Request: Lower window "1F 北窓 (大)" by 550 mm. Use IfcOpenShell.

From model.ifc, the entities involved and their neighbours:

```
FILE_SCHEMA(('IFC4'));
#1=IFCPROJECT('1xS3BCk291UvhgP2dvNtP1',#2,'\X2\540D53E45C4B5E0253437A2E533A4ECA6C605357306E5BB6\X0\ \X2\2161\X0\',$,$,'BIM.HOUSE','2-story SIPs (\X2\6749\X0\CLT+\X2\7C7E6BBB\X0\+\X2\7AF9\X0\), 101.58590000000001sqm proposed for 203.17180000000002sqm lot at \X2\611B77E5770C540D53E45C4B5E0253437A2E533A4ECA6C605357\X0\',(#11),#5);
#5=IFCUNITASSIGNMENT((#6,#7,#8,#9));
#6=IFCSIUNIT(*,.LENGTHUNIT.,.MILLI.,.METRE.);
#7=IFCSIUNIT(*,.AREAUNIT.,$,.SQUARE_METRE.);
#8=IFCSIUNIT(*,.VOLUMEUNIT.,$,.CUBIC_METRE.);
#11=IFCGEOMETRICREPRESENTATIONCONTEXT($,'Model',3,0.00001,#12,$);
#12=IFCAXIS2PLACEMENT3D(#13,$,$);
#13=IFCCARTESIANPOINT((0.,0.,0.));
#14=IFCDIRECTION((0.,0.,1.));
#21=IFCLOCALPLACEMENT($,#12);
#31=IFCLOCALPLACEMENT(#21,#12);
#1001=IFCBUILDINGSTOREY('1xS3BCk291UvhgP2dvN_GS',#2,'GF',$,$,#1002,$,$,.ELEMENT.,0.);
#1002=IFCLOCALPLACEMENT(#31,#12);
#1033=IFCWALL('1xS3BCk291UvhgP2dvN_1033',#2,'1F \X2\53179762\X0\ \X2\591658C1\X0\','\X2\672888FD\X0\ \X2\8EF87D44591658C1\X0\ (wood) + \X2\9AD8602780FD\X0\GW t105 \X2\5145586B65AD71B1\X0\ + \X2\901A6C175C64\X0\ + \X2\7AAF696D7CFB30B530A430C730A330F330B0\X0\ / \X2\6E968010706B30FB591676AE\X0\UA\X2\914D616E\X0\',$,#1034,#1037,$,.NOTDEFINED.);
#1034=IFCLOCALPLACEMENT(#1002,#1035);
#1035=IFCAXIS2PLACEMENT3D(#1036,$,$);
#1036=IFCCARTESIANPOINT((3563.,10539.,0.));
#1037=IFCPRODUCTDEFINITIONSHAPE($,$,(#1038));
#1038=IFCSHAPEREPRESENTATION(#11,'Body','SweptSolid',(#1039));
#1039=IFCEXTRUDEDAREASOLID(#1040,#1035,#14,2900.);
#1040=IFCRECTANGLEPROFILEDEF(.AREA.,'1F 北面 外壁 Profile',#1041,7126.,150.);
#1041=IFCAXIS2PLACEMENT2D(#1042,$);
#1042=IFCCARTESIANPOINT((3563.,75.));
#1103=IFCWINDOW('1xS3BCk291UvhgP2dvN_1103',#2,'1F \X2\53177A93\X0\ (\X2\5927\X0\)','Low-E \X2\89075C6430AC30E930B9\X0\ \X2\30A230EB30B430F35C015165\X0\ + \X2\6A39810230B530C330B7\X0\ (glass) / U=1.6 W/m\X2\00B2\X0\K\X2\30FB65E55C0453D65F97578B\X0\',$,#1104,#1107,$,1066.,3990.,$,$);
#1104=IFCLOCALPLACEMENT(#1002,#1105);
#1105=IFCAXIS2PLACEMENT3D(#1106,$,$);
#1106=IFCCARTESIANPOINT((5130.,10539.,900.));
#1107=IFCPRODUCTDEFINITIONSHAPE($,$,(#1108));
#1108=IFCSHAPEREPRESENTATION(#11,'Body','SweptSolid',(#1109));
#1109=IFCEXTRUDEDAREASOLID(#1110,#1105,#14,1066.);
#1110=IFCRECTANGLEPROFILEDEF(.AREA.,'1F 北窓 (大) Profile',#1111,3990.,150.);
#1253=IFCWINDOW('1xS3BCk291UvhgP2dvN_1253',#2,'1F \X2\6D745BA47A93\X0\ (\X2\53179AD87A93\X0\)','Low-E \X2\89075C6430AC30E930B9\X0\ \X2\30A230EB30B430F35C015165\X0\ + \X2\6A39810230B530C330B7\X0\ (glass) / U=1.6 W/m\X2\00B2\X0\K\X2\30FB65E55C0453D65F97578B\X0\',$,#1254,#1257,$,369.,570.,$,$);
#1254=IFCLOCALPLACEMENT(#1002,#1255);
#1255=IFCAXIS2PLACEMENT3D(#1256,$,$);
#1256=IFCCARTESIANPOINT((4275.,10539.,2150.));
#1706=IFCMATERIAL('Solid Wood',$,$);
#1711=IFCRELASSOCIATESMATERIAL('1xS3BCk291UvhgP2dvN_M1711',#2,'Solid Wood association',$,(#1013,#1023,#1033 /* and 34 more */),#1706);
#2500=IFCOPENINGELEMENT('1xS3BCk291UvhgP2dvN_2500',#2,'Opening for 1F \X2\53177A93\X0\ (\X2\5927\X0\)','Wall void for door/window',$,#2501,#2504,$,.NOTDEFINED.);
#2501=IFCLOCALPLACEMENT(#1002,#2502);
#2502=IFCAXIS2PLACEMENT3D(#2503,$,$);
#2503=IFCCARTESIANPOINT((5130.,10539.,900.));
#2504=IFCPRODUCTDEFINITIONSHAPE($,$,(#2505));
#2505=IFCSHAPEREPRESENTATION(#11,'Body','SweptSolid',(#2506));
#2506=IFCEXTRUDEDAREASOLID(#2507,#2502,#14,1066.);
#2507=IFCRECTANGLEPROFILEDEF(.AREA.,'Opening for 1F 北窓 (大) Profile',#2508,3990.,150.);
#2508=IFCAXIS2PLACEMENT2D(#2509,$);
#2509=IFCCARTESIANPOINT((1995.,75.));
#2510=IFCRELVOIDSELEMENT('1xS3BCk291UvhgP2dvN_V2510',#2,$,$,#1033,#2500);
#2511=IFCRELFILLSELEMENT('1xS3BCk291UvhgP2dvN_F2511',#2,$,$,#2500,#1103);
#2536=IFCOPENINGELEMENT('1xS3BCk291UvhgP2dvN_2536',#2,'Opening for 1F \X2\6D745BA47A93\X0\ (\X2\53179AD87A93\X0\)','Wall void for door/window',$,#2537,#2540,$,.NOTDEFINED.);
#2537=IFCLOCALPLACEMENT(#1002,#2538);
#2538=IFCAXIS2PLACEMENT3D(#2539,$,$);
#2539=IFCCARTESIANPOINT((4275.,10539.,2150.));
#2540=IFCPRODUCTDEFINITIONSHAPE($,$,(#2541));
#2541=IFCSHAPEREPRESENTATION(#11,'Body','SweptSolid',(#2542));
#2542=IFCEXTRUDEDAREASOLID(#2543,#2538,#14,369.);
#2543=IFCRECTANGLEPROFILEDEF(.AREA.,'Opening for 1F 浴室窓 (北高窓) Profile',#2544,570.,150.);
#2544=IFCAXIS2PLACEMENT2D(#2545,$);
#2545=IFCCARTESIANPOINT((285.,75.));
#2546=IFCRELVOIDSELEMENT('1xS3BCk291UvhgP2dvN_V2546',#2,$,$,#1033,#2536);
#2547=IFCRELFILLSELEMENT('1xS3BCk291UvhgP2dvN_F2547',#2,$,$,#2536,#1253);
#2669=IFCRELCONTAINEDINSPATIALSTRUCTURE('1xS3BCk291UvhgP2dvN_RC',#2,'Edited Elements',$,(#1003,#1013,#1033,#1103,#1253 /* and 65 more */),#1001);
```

```python
import numpy as np
import ifcopenshell
import ifcopenshell.api.geometry
import ifcopenshell.util.placement
import ifcopenshell.util.unit

model = ifcopenshell.open("model.ifc")
unit_scale = ifcopenshell.util.unit.calculate_unit_scale(model)

window = model.by_guid("1xS3BCk291UvhgP2dvN_1103")
opening = window.FillsVoids[0].RelatingOpeningElement
dz = -0.55 / unit_scale

shift = np.array([0.0, 0.0, dz])
# The window is not placed relative to its opening, so move both.
for product in (opening, window):
    matrix = ifcopenshell.util.placement.get_local_placement(product.ObjectPlacement)
    matrix[:3, 3] += shift
    ifcopenshell.api.geometry.edit_object_placement(model, product=product, matrix=matrix, is_si=False)

print(f"moved by {dz * unit_scale:+.3f} m")

model.write("model_updated.ifc")
```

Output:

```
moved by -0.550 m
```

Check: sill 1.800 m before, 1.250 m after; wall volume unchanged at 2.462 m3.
